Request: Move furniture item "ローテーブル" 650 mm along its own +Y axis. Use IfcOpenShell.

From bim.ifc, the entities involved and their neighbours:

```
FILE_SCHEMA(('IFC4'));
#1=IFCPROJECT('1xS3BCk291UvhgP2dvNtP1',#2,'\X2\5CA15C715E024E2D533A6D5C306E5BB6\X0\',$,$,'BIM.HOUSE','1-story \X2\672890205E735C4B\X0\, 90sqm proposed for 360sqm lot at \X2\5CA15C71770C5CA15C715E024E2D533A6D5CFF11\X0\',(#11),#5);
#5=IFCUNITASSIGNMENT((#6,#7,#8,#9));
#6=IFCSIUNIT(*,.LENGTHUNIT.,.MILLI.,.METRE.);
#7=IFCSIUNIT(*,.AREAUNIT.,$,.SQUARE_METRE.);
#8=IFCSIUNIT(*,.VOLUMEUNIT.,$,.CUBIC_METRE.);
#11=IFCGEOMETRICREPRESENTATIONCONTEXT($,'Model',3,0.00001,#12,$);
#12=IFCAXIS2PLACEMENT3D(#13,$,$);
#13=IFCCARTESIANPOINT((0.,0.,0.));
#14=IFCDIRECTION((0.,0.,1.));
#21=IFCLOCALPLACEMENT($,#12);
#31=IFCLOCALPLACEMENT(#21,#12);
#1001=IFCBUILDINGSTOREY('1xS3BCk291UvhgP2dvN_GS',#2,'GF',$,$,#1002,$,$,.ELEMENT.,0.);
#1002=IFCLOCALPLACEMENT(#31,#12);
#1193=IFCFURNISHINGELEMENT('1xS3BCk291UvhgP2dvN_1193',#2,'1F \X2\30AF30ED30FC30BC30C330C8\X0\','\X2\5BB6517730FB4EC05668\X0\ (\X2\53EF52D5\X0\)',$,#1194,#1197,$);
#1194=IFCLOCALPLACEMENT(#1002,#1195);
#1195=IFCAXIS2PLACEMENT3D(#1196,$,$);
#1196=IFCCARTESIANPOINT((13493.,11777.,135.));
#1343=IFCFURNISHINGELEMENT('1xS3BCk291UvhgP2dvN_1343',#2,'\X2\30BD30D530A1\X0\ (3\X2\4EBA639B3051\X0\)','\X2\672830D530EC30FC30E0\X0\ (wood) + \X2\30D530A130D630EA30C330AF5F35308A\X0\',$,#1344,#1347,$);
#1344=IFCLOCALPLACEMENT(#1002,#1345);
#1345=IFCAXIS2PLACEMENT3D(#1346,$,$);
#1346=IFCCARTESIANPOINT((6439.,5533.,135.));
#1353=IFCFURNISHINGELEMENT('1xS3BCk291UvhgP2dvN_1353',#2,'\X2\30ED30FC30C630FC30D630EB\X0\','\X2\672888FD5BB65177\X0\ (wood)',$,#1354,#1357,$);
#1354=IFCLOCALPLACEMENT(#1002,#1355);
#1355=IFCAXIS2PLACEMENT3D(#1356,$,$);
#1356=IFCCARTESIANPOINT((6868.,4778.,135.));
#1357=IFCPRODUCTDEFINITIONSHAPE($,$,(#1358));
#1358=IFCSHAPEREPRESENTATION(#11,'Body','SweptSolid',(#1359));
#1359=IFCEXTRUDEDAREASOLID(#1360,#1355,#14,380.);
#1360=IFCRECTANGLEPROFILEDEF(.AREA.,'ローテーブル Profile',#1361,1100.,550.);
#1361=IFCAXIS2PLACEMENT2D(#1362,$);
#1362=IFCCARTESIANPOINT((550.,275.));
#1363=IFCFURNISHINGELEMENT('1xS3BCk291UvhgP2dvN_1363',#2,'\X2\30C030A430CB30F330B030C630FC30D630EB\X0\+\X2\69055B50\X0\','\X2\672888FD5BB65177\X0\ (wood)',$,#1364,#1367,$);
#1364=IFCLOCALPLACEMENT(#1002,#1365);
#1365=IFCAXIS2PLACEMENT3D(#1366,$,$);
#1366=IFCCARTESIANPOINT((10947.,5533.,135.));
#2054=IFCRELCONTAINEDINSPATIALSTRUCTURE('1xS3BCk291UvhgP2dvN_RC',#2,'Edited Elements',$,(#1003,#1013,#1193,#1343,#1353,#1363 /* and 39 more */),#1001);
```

```python
import ifcopenshell
import ifcopenshell.api.geometry
import ifcopenshell.util.placement
import ifcopenshell.util.unit

model = ifcopenshell.open("bim.ifc")
unit_scale = ifcopenshell.util.unit.calculate_unit_scale(model)

item = model.by_guid("1xS3BCk291UvhgP2dvN_1353")
matrix = ifcopenshell.util.placement.get_local_placement(item.ObjectPlacement)
matrix[:3, 3] += matrix[:3, 1] * 0.65 / unit_scale
ifcopenshell.api.geometry.edit_object_placement(model, product=item, matrix=matrix, is_si=False)

print(ifcopenshell.util.placement.get_local_placement(item.ObjectPlacement).round(3) + 0.0)

model.write("bim_updated.ifc")
```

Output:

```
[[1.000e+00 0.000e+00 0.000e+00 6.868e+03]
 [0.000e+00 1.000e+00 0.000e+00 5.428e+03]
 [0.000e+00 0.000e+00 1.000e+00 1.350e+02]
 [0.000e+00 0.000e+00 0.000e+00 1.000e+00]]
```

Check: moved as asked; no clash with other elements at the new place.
